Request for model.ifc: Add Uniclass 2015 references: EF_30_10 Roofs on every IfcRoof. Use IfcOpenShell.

First a look at what the model holds.

```python
import ifcopenshell

model = ifcopenshell.open("model.ifc")
print(model.schema)
print("classifications:", [c.Name for c in model.by_type("IfcClassification")])
for ifc_class in ("IfcDoor", "IfcRoof", "IfcStair", "IfcWall", "IfcWindow"):
    print(ifc_class, len(model.by_type(ifc_class)))
```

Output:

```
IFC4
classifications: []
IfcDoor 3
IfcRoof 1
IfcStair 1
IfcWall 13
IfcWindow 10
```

```python
import ifcopenshell
import ifcopenshell.api.classification

model = ifcopenshell.open("model.ifc")

system = ifcopenshell.api.classification.add_classification(model, classification="Uniclass 2015")

codes = {
    "IfcRoof": ("EF_30_10", "Roofs"),
}
for ifc_class, (code, name) in codes.items():
    products = model.by_type(ifc_class)
    ifcopenshell.api.classification.add_reference(
        model, products=products, classification=system, identification=code, name=name
    )
    print(code, len(products))

model.write("model_updated.ifc")
```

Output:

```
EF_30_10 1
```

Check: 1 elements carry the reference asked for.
